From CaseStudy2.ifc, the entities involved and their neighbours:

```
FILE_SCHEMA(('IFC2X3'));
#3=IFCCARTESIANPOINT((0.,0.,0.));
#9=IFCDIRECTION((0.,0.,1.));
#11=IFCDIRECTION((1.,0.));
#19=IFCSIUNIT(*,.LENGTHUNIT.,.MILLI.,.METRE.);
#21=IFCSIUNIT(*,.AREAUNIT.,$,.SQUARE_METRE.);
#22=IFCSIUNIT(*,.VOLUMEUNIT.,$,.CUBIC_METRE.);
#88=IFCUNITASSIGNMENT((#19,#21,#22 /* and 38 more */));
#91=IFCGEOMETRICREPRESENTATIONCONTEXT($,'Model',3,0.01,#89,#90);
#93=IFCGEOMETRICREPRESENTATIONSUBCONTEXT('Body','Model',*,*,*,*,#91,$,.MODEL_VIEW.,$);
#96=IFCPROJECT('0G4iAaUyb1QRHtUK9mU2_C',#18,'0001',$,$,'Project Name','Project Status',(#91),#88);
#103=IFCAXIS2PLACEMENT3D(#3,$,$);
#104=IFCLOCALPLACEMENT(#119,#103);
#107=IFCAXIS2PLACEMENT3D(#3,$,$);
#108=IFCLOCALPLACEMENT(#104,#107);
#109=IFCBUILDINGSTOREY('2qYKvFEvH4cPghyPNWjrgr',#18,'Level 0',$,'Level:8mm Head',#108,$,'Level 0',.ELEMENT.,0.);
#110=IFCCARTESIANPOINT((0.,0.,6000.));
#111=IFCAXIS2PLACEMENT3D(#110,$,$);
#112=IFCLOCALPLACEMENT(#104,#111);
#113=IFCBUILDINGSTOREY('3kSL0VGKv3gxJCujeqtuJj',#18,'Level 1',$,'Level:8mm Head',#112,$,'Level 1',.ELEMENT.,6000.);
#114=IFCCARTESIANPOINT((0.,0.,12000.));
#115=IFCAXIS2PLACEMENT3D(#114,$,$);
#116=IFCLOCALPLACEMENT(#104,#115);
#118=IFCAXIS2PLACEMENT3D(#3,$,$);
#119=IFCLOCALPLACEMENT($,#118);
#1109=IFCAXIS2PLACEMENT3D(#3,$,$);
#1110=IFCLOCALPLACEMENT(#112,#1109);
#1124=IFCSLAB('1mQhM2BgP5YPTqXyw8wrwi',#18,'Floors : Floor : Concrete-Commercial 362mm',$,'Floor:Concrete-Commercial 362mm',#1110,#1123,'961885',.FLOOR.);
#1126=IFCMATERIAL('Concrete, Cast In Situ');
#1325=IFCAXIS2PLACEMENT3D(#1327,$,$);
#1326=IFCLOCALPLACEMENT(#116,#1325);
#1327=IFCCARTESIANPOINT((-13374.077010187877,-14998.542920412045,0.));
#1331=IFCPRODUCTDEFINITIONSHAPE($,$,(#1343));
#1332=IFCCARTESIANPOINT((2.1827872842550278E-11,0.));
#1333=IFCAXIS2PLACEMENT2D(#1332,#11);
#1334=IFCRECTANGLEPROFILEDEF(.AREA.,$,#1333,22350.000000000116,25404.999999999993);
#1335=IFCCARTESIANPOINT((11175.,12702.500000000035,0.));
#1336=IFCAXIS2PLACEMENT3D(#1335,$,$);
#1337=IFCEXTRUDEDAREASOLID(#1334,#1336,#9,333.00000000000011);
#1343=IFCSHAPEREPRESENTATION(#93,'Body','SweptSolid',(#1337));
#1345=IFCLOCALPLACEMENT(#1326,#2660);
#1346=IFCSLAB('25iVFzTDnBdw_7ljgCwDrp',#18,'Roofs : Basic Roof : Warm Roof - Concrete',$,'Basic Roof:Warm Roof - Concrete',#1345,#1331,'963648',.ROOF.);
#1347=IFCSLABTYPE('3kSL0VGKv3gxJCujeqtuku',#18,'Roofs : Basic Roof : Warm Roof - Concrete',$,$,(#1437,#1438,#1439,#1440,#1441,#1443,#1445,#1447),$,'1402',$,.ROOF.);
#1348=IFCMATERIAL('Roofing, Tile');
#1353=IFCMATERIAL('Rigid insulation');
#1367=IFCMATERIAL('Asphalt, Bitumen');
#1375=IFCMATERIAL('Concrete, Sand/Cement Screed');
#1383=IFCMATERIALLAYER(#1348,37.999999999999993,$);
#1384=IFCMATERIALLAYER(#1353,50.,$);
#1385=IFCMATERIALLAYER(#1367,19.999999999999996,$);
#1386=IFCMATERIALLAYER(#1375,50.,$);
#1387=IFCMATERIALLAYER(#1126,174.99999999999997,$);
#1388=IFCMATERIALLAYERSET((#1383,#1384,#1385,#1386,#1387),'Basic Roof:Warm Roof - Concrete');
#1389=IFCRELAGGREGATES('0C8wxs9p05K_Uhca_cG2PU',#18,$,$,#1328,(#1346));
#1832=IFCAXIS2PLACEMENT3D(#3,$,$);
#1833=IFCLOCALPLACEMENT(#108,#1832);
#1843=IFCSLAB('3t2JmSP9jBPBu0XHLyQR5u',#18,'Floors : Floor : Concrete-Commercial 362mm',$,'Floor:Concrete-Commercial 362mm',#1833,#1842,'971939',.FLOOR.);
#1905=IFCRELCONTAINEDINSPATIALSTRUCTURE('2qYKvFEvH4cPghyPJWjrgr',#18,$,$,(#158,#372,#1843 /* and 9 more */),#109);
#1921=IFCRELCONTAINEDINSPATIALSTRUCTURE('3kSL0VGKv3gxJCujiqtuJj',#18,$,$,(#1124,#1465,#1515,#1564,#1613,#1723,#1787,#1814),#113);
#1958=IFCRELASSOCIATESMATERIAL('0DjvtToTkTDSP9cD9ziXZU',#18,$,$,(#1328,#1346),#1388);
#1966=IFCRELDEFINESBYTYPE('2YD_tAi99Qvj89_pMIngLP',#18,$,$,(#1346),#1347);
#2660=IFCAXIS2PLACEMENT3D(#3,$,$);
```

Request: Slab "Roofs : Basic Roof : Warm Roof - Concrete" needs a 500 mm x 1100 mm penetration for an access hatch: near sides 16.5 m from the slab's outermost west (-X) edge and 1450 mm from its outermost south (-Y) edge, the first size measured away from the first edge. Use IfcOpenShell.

```python
import numpy as np
import ifcopenshell
import ifcopenshell.api.feature
import ifcopenshell.api.geometry
import ifcopenshell.api.root
import ifcopenshell.geom
import ifcopenshell.util.placement
import ifcopenshell.util.representation
import ifcopenshell.util.shape
import ifcopenshell.util.unit

model = ifcopenshell.open("CaseStudy2.ifc")
unit_scale = ifcopenshell.util.unit.calculate_unit_scale(model)
settings = ifcopenshell.geom.settings()


def volume(element):
    """Net volume in cubic metres, openings subtracted."""
    shape = ifcopenshell.geom.create_shape(settings, element)
    return ifcopenshell.util.shape.get_volume(shape.geometry)


slab = model.by_id(1346)
before = volume(slab)

# Extent in the slab's own axes, in metres. The edges named are its -X and -Y sides.
slab_shape = ifcopenshell.geom.create_shape(settings, slab)
vertices = ifcopenshell.util.shape.get_vertices(slab_shape.geometry)
x_min, y_min, bottom = vertices.min(axis=0)
top = vertices[:, 2].max()

opening = ifcopenshell.api.root.create_entity(model, ifc_class="IfcOpeningElement", name="Access hatch opening")
context = ifcopenshell.util.representation.get_context(model, "Model", "Body", "MODEL_VIEW")
width, depth = 0.5, 1.1
outline = [(0.0, 0.0), (width, 0.0), (width, depth), (0.0, depth), (0.0, 0.0)]
# Overshoot both faces by 50 mm so the cut is clean.
shape = ifcopenshell.api.geometry.add_slab_representation(
    model, context=context, depth=top - bottom + 0.1, polyline=outline
)
ifcopenshell.api.geometry.assign_representation(model, product=opening, representation=shape)

matrix = ifcopenshell.util.placement.get_local_placement(slab.ObjectPlacement)
matrix[:, 3] = matrix @ np.append(np.array([x_min + 16.5, y_min + 1.45, bottom - 0.05]) / unit_scale, 1.0)
ifcopenshell.api.geometry.edit_object_placement(model, product=opening, matrix=matrix, is_si=False)
ifcopenshell.api.feature.add_feature(model, feature=opening, element=slab)

after = volume(slab)

print(f"slab volume {before:.3f} -> {after:.3f} m3")

model.write("CaseStudy2_updated.ifc")
```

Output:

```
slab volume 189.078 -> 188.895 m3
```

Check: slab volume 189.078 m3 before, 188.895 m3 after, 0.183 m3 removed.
